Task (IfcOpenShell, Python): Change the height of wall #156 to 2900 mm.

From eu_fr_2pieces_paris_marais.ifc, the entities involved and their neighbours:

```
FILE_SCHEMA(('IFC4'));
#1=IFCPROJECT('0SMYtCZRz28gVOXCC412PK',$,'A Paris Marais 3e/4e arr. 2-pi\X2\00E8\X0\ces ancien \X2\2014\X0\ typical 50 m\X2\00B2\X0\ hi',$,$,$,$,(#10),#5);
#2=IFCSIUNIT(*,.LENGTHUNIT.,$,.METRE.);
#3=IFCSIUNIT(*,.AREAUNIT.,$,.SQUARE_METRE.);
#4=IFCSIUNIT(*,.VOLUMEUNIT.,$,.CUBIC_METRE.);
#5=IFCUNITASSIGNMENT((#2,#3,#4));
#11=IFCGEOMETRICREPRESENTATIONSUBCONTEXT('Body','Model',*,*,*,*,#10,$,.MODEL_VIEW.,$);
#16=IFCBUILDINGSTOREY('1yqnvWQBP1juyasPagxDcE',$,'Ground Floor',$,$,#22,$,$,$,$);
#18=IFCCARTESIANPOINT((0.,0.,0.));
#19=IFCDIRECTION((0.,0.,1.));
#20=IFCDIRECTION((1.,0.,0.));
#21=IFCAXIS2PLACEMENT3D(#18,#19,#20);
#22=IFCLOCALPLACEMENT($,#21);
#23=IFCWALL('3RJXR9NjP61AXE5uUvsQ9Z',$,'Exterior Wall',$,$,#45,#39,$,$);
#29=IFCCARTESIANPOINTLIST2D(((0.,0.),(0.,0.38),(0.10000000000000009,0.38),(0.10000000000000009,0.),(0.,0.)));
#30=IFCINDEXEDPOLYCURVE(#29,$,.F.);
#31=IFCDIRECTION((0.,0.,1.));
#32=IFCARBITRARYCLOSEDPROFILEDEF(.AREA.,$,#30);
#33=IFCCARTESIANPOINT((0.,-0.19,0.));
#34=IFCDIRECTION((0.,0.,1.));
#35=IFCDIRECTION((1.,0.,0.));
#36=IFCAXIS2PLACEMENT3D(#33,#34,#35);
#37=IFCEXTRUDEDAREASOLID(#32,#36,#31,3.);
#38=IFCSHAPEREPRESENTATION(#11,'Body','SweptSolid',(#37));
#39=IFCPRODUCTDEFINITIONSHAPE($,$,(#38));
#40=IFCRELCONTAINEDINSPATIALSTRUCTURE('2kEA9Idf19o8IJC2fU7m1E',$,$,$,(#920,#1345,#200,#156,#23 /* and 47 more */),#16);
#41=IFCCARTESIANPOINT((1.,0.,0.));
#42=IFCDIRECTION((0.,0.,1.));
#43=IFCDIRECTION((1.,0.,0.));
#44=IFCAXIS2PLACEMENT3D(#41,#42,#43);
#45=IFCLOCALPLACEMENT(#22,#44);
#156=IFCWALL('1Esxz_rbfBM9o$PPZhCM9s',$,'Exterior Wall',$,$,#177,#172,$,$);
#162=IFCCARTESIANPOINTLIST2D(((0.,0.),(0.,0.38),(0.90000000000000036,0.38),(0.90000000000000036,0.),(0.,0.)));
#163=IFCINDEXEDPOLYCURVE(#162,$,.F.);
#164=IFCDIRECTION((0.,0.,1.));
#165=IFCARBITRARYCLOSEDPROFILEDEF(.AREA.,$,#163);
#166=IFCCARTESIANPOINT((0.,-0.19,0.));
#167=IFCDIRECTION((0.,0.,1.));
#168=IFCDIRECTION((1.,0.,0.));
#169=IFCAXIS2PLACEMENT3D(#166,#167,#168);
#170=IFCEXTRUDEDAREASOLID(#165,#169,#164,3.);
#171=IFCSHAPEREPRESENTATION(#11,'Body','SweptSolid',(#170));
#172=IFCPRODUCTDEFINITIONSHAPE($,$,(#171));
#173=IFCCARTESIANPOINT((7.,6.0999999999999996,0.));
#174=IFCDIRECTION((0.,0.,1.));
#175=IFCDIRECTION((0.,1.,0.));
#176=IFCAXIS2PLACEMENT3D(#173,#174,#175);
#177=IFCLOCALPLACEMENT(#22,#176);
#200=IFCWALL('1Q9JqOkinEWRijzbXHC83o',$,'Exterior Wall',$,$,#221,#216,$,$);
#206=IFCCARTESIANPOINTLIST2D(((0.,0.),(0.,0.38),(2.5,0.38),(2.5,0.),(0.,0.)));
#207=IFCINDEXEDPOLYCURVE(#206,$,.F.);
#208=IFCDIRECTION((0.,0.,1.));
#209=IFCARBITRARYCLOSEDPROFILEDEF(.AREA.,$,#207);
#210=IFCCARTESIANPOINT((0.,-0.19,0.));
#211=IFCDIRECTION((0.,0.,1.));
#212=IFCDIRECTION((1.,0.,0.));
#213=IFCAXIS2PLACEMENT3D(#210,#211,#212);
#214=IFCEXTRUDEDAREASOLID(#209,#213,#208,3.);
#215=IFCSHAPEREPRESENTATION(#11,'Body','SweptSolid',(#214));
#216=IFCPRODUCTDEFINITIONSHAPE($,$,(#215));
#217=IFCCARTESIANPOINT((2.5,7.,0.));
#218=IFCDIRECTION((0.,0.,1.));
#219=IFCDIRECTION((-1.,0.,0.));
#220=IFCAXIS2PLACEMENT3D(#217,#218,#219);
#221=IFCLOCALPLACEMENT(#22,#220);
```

```python
import ifcopenshell
import ifcopenshell.geom
import ifcopenshell.util.representation
import ifcopenshell.util.shape
import ifcopenshell.util.unit

model = ifcopenshell.open("eu_fr_2pieces_paris_marais.ifc")
unit_scale = ifcopenshell.util.unit.calculate_unit_scale(model)
settings = ifcopenshell.geom.settings()


def volume(element):
    """Net volume in cubic metres, openings subtracted."""
    shape = ifcopenshell.geom.create_shape(settings, element)
    return ifcopenshell.util.shape.get_volume(shape.geometry)


wall = model.by_id(156)
before = volume(wall)

body = ifcopenshell.util.representation.get_representation(wall, "Model", "Body")
solid = body.Items[0]
old_height = solid.Depth
solid.Depth = 2.9 / unit_scale
after = volume(wall)

print(f"height {old_height:g} -> {solid.Depth:g}, volume {before:.3f} -> {after:.3f} m3")

model.write("eu_fr_2pieces_paris_marais-out.ifc")
```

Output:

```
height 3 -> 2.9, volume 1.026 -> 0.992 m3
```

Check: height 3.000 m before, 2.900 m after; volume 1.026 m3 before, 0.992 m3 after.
